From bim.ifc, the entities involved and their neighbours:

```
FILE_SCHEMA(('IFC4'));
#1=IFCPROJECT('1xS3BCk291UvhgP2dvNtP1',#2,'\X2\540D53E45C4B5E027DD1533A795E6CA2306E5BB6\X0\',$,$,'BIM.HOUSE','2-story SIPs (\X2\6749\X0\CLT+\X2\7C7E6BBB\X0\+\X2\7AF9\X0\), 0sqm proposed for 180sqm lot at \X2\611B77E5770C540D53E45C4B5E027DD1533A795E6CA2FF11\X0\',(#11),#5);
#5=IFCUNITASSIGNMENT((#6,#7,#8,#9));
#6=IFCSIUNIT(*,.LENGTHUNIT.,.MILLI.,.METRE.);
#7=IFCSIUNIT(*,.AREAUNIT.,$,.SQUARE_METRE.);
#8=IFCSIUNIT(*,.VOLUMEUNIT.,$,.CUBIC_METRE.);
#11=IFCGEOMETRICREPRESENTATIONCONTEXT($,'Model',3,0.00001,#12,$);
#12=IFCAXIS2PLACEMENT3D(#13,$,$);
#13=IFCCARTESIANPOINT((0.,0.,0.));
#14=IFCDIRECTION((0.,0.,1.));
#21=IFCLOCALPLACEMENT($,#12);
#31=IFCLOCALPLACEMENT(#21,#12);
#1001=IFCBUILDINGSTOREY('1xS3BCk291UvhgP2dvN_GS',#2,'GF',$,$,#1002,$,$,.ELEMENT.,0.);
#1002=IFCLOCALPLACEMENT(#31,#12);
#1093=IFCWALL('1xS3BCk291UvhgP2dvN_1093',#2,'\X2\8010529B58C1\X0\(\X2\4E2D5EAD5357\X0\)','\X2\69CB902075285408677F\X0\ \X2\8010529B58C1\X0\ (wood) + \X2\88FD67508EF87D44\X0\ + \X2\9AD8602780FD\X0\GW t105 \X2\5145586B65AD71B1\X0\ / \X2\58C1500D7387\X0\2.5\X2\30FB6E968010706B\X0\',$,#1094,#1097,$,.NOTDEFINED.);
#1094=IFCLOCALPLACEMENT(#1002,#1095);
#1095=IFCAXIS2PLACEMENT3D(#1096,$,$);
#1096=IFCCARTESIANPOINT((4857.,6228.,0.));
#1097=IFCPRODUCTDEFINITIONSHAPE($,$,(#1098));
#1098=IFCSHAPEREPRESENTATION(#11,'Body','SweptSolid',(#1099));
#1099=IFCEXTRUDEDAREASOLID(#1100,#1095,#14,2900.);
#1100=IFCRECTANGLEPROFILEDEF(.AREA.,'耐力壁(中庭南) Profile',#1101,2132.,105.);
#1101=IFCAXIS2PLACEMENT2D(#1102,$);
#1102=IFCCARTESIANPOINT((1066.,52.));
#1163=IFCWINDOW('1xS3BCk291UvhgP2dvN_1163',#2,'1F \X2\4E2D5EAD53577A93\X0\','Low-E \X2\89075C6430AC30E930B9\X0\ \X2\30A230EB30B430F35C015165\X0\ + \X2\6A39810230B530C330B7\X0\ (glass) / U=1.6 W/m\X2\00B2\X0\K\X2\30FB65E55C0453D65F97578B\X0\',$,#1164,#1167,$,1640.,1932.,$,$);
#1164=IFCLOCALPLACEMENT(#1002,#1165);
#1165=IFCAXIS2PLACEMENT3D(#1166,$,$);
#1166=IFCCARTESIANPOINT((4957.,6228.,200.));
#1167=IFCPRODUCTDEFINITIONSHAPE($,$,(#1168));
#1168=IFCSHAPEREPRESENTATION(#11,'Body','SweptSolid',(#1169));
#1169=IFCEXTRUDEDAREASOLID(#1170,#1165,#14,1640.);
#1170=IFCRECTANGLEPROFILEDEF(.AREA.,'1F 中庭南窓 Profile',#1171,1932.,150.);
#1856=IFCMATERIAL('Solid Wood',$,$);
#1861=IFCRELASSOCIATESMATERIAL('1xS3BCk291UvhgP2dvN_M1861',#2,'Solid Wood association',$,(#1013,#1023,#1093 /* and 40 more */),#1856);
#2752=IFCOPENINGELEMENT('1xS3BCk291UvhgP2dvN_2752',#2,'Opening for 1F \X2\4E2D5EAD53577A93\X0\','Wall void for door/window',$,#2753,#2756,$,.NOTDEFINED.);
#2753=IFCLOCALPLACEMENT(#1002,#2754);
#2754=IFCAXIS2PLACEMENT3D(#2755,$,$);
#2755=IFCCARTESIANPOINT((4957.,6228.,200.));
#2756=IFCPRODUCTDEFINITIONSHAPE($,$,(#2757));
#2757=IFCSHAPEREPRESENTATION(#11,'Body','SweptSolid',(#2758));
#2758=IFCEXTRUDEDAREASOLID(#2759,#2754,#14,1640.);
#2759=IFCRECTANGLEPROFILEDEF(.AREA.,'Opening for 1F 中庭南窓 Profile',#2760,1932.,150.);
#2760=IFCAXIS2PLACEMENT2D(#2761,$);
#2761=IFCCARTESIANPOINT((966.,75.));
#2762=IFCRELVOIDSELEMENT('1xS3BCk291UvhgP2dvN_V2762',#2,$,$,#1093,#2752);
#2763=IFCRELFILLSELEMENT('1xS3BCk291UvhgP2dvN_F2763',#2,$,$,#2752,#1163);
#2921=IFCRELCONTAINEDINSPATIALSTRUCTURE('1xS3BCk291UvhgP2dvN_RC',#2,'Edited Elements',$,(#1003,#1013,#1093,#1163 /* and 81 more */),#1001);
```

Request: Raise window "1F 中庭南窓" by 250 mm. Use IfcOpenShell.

```python
import numpy as np
import ifcopenshell
import ifcopenshell.api.geometry
import ifcopenshell.util.placement
import ifcopenshell.util.unit

model = ifcopenshell.open("bim.ifc")
unit_scale = ifcopenshell.util.unit.calculate_unit_scale(model)

window = model.by_guid("1xS3BCk291UvhgP2dvN_1163")
opening = window.FillsVoids[0].RelatingOpeningElement
dz = 250.0

shift = np.array([0.0, 0.0, dz])
# The window is not placed relative to its opening, so move both.
for product in (opening, window):
    matrix = ifcopenshell.util.placement.get_local_placement(product.ObjectPlacement)
    matrix[:3, 3] += shift
    ifcopenshell.api.geometry.edit_object_placement(model, product=product, matrix=matrix, is_si=False)

print(f"moved by {dz * unit_scale:+.3f} m")

model.write("bim_v2.ifc")
```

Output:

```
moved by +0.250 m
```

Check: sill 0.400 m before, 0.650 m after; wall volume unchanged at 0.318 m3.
